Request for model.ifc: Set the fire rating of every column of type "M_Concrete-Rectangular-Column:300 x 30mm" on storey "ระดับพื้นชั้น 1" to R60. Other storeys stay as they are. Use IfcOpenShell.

First a look at what the model holds.

```python
import ifcopenshell
import ifcopenshell.util.element

model = ifcopenshell.open("model.ifc")
print(model.schema)
storey = next(s for s in model.by_type("IfcBuildingStorey") if s.Name == "ระดับพื้นชั้น 1")
columns = [e for e in ifcopenshell.util.element.get_decomposition(storey) if e.is_a("IfcColumn")]
seen = {}
for e in columns:
    element_type = ifcopenshell.util.element.get_type(e)
    key = (element_type.Name if element_type != e and element_type else None, ifcopenshell.util.element.get_pset(e, "Pset_ColumnCommon", "FireRating"))
    seen[key] = seen.get(key, 0) + 1
for (name, value), count in sorted(seen.items(), key=str):
    print(count, "x", name, "|", value)
```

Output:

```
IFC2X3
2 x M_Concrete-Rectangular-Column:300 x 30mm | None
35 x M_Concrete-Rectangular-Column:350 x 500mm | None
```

```python
import ifcopenshell
import ifcopenshell.api.pset
import ifcopenshell.util.element

model = ifcopenshell.open("model.ifc")

storey = next(s for s in model.by_type("IfcBuildingStorey") if s.Name == "ระดับพื้นชั้น 1")
columns = [e for e in ifcopenshell.util.element.get_decomposition(storey) if e.is_a("IfcColumn")]

count = 0
for e in columns:
    element_type = ifcopenshell.util.element.get_type(e)
    if element_type in (None, e) or element_type.Name != "M_Concrete-Rectangular-Column:300 x 30mm":
        continue
    # add_pset returns the element's existing set when there is one.
    pset = ifcopenshell.api.pset.add_pset(model, product=e, name="Pset_ColumnCommon")
    ifcopenshell.api.pset.edit_pset(model, pset=pset, properties={"FireRating": "R60"})
    count += 1

print(count, "columns updated")

model.write("model-out.ifc")
```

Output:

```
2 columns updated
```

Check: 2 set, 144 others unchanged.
